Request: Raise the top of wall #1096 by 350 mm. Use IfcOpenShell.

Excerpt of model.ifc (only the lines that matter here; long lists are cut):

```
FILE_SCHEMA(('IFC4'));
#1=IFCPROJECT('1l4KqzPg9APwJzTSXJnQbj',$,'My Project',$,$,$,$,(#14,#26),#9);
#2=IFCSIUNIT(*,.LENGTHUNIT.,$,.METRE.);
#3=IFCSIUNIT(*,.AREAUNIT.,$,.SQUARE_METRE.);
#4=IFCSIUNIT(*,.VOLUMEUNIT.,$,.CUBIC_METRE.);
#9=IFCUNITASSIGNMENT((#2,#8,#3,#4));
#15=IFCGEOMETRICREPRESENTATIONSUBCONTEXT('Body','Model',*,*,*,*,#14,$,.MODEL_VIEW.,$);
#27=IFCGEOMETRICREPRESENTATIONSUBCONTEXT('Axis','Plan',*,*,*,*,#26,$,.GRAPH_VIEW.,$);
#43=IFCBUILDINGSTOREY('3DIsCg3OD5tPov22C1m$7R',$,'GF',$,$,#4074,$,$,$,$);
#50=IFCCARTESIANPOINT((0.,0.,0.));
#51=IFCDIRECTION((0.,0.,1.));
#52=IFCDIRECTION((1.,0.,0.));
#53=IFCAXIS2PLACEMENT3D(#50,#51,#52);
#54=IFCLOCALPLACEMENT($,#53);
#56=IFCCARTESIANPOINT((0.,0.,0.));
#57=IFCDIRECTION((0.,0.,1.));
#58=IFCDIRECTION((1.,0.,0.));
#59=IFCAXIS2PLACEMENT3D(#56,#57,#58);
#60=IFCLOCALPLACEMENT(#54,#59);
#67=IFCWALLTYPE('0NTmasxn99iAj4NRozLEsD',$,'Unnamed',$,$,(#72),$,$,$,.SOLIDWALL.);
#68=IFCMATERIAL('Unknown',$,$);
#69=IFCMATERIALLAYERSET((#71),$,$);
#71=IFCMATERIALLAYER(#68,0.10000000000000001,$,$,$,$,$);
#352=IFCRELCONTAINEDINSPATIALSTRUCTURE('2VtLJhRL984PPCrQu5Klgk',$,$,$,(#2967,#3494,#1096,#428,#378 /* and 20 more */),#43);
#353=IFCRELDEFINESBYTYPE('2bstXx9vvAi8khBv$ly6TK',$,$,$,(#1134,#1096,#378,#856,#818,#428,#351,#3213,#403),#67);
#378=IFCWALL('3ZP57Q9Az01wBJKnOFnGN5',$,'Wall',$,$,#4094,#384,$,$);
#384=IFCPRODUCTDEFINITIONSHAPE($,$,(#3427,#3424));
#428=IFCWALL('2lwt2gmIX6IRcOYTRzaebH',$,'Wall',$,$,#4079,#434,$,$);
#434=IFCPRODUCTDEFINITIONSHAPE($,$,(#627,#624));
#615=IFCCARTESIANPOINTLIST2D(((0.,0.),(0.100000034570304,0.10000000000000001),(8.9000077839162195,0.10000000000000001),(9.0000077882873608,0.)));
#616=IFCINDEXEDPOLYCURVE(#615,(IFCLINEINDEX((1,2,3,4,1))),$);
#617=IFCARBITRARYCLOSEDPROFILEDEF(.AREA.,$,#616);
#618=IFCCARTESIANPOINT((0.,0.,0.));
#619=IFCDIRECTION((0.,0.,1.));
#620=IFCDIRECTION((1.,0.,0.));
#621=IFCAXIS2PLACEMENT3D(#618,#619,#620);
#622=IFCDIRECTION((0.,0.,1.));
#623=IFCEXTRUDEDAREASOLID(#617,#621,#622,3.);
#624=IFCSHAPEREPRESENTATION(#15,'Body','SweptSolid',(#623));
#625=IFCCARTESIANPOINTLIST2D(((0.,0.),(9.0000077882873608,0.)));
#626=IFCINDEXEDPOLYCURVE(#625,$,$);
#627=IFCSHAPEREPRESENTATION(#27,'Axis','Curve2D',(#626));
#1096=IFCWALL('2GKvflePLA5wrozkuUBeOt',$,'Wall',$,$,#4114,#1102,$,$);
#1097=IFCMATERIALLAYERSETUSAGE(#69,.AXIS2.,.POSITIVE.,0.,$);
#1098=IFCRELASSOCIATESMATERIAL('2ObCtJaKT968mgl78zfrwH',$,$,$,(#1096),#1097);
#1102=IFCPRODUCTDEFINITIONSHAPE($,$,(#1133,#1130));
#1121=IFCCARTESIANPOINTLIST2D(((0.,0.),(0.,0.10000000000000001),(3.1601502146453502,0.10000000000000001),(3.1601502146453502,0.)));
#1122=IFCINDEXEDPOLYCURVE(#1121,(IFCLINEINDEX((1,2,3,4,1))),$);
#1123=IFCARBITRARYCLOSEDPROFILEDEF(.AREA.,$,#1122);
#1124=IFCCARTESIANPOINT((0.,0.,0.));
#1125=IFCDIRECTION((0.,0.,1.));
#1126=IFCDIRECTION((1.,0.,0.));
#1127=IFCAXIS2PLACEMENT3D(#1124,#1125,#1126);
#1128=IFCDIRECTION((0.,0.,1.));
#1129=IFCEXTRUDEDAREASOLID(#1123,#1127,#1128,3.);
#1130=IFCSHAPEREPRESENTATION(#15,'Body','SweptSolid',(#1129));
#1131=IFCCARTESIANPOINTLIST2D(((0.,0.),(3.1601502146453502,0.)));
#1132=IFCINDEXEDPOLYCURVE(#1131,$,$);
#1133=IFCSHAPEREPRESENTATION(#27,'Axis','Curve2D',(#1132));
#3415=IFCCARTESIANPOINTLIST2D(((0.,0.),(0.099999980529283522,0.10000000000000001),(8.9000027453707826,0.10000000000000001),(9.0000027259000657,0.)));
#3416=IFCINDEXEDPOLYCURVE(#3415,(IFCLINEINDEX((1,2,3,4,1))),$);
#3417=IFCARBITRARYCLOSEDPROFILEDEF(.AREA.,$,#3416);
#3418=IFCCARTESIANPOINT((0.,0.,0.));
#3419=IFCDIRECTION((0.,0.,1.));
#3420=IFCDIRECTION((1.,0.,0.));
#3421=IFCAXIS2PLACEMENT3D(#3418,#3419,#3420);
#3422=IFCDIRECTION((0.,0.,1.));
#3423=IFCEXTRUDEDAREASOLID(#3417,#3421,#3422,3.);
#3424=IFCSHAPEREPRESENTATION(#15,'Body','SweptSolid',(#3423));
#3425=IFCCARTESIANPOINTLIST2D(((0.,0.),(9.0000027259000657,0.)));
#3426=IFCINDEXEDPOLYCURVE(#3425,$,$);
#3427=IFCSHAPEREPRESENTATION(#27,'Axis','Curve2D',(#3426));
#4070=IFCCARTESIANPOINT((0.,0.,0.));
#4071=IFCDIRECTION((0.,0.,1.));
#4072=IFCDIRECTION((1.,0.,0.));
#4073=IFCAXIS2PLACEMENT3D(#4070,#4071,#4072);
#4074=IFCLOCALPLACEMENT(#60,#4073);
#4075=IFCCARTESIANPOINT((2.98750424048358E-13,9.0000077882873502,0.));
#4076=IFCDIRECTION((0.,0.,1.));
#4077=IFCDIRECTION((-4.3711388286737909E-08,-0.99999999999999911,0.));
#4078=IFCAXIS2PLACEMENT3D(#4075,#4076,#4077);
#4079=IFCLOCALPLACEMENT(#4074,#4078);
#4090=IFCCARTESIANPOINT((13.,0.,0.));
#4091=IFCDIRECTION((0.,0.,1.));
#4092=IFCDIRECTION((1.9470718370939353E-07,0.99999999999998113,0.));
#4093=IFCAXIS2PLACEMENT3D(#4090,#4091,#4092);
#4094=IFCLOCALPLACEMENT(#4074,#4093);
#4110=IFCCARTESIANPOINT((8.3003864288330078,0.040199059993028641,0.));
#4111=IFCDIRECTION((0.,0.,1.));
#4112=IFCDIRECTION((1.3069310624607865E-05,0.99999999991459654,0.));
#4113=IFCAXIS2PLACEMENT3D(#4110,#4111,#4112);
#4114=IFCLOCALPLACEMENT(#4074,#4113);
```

```python
import ifcopenshell
import ifcopenshell.geom
import ifcopenshell.util.representation
import ifcopenshell.util.shape
import ifcopenshell.util.unit

model = ifcopenshell.open("model.ifc")
unit_scale = ifcopenshell.util.unit.calculate_unit_scale(model)
settings = ifcopenshell.geom.settings()


def volume(element):
    """Net volume in cubic metres, openings subtracted."""
    shape = ifcopenshell.geom.create_shape(settings, element)
    return ifcopenshell.util.shape.get_volume(shape.geometry)


wall = model.by_id(1096)
before = volume(wall)

body = ifcopenshell.util.representation.get_representation(wall, "Model", "Body")
solid = body.Items[0]
old_height = solid.Depth
solid.Depth += 0.35 / unit_scale
after = volume(wall)

print(f"height {old_height:g} -> {solid.Depth:g}, volume {before:.3f} -> {after:.3f} m3")

model.write("model_updated.ifc")
```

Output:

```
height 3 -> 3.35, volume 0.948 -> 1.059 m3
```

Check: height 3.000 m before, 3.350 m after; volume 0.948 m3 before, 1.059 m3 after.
